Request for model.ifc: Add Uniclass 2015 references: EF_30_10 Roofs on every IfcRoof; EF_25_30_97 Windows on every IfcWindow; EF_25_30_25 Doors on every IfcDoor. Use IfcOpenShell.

First a look at what the model holds.

```python
import ifcopenshell

model = ifcopenshell.open("model.ifc")
print(model.schema)
print("classifications:", [c.Name for c in model.by_type("IfcClassification")])
for ifc_class in ("IfcDoor", "IfcRoof", "IfcStair", "IfcWall", "IfcWindow"):
    print(ifc_class, len(model.by_type(ifc_class)))
```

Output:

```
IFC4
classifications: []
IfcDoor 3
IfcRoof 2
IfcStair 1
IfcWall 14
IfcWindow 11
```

```python
import ifcopenshell
import ifcopenshell.api.classification

model = ifcopenshell.open("model.ifc")

system = ifcopenshell.api.classification.add_classification(model, classification="Uniclass 2015")

codes = {
    "IfcRoof": ("EF_30_10", "Roofs"),
    "IfcWindow": ("EF_25_30_97", "Windows"),
    "IfcDoor": ("EF_25_30_25", "Doors"),
}
for ifc_class, (code, name) in codes.items():
    products = model.by_type(ifc_class)
    ifcopenshell.api.classification.add_reference(
        model, products=products, classification=system, identification=code, name=name
    )
    print(code, len(products))

model.write("model_updated.ifc")
```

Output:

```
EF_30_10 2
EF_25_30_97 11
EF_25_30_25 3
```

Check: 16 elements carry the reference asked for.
